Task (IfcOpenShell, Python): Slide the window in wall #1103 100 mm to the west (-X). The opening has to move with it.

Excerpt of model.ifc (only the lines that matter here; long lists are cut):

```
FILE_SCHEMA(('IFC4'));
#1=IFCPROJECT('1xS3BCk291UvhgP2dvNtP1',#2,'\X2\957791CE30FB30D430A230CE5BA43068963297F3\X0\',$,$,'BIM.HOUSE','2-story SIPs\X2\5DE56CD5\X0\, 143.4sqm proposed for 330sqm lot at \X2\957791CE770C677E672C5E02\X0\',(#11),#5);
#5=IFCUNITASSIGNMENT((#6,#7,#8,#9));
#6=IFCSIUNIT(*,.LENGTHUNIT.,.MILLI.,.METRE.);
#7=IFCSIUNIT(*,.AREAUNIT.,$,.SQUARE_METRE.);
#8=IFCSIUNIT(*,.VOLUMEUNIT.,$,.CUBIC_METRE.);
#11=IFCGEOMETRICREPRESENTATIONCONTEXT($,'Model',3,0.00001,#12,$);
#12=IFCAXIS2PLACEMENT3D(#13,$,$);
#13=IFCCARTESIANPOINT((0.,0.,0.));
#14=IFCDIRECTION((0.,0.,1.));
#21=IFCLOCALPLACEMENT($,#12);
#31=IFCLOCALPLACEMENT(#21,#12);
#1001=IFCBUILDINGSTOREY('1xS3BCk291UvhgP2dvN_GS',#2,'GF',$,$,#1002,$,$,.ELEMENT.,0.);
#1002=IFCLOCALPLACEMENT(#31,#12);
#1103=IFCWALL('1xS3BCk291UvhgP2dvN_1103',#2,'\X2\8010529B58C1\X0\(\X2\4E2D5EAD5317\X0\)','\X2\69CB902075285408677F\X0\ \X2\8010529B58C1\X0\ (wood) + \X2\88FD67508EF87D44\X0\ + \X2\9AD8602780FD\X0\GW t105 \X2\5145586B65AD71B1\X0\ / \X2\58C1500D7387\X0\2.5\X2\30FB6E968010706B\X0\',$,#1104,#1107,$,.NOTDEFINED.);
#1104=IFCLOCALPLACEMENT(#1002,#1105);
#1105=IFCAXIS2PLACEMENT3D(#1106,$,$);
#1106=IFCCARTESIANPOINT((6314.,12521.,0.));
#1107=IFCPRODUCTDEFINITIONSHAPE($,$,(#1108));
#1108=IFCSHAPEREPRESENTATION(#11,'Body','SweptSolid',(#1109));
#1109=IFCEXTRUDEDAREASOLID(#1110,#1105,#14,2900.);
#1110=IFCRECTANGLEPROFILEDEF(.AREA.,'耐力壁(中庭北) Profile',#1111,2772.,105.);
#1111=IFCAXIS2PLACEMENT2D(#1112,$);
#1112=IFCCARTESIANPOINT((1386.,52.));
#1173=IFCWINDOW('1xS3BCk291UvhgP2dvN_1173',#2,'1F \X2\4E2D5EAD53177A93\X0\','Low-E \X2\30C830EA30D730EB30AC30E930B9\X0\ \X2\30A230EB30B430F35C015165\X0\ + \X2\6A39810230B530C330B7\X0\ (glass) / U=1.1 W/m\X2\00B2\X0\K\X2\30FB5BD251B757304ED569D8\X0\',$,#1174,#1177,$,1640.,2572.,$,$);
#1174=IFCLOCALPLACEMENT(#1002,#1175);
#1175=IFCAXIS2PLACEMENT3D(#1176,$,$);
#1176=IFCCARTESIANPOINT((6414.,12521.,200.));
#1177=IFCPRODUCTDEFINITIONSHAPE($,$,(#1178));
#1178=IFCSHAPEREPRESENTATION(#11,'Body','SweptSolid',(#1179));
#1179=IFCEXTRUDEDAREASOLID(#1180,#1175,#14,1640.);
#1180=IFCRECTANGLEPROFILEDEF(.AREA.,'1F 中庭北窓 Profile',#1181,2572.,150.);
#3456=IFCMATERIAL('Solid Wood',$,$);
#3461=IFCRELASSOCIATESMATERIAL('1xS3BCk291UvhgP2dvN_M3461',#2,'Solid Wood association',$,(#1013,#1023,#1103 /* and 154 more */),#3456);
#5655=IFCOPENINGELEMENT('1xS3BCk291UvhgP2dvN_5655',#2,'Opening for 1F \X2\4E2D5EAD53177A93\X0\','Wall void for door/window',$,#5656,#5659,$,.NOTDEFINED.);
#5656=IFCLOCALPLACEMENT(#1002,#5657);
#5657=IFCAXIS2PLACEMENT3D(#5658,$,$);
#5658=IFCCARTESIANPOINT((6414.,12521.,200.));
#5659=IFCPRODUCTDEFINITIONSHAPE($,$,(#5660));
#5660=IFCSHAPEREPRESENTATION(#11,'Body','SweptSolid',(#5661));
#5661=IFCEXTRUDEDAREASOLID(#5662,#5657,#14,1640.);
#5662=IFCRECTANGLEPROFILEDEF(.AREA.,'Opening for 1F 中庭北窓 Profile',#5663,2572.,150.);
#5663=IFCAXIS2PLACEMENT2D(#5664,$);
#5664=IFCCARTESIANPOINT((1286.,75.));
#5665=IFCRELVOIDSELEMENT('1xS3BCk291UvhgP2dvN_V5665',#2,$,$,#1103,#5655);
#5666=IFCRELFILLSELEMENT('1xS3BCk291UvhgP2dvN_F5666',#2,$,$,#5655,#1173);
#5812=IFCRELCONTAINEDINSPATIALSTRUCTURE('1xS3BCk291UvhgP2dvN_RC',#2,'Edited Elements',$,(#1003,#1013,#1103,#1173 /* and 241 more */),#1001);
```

```python
import ifcopenshell
import ifcopenshell.api.geometry
import ifcopenshell.util.placement
import ifcopenshell.util.unit

model = ifcopenshell.open("model.ifc")
unit_scale = ifcopenshell.util.unit.calculate_unit_scale(model)

window = model.by_guid("1xS3BCk291UvhgP2dvN_1173")
opening = window.FillsVoids[0].RelatingOpeningElement
wall = opening.VoidsElements[0].RelatingBuildingElement

wall_matrix = ifcopenshell.util.placement.get_local_placement(wall.ObjectPlacement)
shift = wall_matrix[:3, 0] * -0.1 / unit_scale
before = ifcopenshell.util.placement.get_local_placement(window.ObjectPlacement)[:3, 3].copy()

# The window is not placed relative to its opening, so move both.
for product in (opening, window):
    matrix = ifcopenshell.util.placement.get_local_placement(product.ObjectPlacement)
    matrix[:3, 3] += shift
    ifcopenshell.api.geometry.edit_object_placement(model, product=product, matrix=matrix, is_si=False)

after = ifcopenshell.util.placement.get_local_placement(window.ObjectPlacement)[:3, 3]
print("window moved by", (after - before).round(3) + 0.0)

model.write("model-out.ifc")
```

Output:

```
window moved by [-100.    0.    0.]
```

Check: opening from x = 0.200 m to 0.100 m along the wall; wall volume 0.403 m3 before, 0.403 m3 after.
